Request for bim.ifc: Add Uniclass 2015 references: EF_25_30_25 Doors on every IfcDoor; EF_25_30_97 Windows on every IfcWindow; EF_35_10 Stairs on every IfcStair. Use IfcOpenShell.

First a look at what the model holds.

```python
import ifcopenshell

model = ifcopenshell.open("bim.ifc")
print(model.schema)
print("classifications:", [c.Name for c in model.by_type("IfcClassification")])
for ifc_class in ("IfcDoor", "IfcRoof", "IfcStair", "IfcWall", "IfcWindow"):
    print(ifc_class, len(model.by_type(ifc_class)))
```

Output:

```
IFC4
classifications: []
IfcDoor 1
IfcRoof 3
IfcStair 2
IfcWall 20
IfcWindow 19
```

```python
import ifcopenshell
import ifcopenshell.api.classification

model = ifcopenshell.open("bim.ifc")

system = ifcopenshell.api.classification.add_classification(model, classification="Uniclass 2015")

codes = {
    "IfcDoor": ("EF_25_30_25", "Doors"),
    "IfcWindow": ("EF_25_30_97", "Windows"),
    "IfcStair": ("EF_35_10", "Stairs"),
}
for ifc_class, (code, name) in codes.items():
    products = model.by_type(ifc_class)
    ifcopenshell.api.classification.add_reference(
        model, products=products, classification=system, identification=code, name=name
    )
    print(code, len(products))

model.write("bim_updated.ifc")
```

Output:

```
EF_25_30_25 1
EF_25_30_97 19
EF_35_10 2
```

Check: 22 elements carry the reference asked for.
